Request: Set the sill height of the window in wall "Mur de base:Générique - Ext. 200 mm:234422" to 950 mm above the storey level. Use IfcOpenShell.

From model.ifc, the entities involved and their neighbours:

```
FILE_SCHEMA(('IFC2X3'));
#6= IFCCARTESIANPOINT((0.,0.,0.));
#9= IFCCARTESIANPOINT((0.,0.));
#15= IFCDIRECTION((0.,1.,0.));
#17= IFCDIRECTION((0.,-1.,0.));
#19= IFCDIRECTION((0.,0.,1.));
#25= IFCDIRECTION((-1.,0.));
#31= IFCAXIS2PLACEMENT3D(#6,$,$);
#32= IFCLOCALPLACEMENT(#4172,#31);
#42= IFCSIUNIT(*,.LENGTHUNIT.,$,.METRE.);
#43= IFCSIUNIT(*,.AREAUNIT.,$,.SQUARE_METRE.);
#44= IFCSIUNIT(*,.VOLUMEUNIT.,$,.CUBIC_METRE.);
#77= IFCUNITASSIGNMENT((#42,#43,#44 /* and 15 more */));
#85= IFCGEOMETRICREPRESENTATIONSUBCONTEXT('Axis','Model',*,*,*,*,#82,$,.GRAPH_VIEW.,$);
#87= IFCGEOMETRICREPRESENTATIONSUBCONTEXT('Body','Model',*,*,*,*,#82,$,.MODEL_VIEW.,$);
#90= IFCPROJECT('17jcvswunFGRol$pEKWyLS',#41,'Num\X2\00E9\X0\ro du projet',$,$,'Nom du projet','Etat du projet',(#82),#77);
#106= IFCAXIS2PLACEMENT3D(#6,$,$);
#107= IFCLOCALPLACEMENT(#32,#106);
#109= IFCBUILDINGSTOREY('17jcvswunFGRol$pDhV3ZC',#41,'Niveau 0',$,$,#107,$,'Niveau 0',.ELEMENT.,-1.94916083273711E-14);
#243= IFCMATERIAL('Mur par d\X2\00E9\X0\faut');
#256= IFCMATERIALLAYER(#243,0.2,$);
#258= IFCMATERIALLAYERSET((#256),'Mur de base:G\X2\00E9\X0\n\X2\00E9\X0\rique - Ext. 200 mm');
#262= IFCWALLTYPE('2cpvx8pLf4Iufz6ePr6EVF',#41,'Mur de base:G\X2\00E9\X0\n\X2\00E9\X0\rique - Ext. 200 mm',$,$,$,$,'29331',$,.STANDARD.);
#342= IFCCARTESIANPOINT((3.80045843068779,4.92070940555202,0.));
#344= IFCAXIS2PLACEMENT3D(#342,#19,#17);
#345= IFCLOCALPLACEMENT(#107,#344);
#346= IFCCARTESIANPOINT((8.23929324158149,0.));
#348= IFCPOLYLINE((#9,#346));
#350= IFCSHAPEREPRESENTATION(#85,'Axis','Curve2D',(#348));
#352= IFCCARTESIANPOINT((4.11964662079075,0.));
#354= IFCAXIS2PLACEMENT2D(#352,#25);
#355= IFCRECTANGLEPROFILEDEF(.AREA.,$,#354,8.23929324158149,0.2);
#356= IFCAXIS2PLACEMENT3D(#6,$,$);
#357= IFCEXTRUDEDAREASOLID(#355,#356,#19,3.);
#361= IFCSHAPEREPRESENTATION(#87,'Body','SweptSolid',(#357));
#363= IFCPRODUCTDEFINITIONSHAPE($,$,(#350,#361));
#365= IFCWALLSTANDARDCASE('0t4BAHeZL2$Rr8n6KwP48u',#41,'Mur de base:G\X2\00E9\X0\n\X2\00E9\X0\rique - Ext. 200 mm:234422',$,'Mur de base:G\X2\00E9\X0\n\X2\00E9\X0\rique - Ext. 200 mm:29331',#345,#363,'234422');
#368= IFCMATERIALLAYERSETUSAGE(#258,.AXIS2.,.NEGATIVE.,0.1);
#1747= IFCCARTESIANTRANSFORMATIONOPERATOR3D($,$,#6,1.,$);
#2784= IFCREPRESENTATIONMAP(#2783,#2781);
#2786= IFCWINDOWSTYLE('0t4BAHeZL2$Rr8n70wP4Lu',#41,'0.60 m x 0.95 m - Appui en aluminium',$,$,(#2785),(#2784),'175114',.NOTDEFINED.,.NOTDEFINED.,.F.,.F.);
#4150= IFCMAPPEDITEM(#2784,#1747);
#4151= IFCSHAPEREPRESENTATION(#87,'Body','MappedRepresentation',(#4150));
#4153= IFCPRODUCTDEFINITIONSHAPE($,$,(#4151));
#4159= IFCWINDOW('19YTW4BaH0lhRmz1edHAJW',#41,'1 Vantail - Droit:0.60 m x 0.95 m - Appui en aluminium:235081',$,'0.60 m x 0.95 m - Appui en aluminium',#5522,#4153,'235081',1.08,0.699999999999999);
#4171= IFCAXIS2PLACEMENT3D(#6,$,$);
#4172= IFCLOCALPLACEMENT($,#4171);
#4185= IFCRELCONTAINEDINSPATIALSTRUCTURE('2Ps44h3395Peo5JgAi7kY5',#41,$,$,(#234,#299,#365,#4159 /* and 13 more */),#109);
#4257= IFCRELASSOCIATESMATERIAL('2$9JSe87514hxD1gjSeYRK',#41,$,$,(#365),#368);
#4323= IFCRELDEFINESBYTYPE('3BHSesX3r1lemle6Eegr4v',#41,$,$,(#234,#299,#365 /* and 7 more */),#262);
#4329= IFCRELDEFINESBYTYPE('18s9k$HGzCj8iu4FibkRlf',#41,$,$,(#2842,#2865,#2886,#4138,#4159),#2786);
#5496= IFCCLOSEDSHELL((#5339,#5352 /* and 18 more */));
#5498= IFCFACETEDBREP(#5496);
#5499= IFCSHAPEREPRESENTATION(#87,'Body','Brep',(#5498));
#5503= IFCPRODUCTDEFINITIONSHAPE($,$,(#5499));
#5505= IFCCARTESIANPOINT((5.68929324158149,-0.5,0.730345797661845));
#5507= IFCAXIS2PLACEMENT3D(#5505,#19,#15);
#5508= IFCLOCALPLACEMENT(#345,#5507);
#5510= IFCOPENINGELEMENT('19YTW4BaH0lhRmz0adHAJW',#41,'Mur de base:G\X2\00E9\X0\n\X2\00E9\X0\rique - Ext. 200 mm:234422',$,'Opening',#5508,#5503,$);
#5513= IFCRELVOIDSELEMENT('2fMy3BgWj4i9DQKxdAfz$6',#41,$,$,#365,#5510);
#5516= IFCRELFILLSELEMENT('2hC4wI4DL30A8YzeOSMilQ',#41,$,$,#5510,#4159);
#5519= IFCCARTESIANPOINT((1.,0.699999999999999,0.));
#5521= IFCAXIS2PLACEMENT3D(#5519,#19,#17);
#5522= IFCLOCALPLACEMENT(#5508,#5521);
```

```python
import numpy as np
import ifcopenshell
import ifcopenshell.api.geometry
import ifcopenshell.geom
import ifcopenshell.util.element
import ifcopenshell.util.placement
import ifcopenshell.util.shape
import ifcopenshell.util.unit

model = ifcopenshell.open("model.ifc")
unit_scale = ifcopenshell.util.unit.calculate_unit_scale(model)

window = model.by_id(4159)
opening = window.FillsVoids[0].RelatingOpeningElement
storey = ifcopenshell.util.element.get_container(window, ifc_class="IfcBuildingStorey")
level = ifcopenshell.util.placement.get_local_placement(storey.ObjectPlacement)[2, 3]

# The opening's origin need not be at the sill, so measure its lowest point.
shape = ifcopenshell.geom.create_shape(ifcopenshell.geom.settings(), opening)
bottom = ifcopenshell.util.shape.get_shape_bottom_elevation(shape, shape.geometry) / unit_scale
dz = level + 0.95 / unit_scale - bottom

shift = np.array([0.0, 0.0, dz])
# The window is placed relative to its opening, so it follows when the opening moves.
matrix = ifcopenshell.util.placement.get_local_placement(opening.ObjectPlacement)
matrix[:3, 3] += shift
ifcopenshell.api.geometry.edit_object_placement(
    model, product=opening, matrix=matrix, is_si=False, should_transform_children=True
)

print(f"moved by {dz * unit_scale:+.3f} m")

model.write("model-out.ifc")
```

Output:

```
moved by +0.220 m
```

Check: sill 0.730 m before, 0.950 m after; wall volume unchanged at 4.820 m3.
